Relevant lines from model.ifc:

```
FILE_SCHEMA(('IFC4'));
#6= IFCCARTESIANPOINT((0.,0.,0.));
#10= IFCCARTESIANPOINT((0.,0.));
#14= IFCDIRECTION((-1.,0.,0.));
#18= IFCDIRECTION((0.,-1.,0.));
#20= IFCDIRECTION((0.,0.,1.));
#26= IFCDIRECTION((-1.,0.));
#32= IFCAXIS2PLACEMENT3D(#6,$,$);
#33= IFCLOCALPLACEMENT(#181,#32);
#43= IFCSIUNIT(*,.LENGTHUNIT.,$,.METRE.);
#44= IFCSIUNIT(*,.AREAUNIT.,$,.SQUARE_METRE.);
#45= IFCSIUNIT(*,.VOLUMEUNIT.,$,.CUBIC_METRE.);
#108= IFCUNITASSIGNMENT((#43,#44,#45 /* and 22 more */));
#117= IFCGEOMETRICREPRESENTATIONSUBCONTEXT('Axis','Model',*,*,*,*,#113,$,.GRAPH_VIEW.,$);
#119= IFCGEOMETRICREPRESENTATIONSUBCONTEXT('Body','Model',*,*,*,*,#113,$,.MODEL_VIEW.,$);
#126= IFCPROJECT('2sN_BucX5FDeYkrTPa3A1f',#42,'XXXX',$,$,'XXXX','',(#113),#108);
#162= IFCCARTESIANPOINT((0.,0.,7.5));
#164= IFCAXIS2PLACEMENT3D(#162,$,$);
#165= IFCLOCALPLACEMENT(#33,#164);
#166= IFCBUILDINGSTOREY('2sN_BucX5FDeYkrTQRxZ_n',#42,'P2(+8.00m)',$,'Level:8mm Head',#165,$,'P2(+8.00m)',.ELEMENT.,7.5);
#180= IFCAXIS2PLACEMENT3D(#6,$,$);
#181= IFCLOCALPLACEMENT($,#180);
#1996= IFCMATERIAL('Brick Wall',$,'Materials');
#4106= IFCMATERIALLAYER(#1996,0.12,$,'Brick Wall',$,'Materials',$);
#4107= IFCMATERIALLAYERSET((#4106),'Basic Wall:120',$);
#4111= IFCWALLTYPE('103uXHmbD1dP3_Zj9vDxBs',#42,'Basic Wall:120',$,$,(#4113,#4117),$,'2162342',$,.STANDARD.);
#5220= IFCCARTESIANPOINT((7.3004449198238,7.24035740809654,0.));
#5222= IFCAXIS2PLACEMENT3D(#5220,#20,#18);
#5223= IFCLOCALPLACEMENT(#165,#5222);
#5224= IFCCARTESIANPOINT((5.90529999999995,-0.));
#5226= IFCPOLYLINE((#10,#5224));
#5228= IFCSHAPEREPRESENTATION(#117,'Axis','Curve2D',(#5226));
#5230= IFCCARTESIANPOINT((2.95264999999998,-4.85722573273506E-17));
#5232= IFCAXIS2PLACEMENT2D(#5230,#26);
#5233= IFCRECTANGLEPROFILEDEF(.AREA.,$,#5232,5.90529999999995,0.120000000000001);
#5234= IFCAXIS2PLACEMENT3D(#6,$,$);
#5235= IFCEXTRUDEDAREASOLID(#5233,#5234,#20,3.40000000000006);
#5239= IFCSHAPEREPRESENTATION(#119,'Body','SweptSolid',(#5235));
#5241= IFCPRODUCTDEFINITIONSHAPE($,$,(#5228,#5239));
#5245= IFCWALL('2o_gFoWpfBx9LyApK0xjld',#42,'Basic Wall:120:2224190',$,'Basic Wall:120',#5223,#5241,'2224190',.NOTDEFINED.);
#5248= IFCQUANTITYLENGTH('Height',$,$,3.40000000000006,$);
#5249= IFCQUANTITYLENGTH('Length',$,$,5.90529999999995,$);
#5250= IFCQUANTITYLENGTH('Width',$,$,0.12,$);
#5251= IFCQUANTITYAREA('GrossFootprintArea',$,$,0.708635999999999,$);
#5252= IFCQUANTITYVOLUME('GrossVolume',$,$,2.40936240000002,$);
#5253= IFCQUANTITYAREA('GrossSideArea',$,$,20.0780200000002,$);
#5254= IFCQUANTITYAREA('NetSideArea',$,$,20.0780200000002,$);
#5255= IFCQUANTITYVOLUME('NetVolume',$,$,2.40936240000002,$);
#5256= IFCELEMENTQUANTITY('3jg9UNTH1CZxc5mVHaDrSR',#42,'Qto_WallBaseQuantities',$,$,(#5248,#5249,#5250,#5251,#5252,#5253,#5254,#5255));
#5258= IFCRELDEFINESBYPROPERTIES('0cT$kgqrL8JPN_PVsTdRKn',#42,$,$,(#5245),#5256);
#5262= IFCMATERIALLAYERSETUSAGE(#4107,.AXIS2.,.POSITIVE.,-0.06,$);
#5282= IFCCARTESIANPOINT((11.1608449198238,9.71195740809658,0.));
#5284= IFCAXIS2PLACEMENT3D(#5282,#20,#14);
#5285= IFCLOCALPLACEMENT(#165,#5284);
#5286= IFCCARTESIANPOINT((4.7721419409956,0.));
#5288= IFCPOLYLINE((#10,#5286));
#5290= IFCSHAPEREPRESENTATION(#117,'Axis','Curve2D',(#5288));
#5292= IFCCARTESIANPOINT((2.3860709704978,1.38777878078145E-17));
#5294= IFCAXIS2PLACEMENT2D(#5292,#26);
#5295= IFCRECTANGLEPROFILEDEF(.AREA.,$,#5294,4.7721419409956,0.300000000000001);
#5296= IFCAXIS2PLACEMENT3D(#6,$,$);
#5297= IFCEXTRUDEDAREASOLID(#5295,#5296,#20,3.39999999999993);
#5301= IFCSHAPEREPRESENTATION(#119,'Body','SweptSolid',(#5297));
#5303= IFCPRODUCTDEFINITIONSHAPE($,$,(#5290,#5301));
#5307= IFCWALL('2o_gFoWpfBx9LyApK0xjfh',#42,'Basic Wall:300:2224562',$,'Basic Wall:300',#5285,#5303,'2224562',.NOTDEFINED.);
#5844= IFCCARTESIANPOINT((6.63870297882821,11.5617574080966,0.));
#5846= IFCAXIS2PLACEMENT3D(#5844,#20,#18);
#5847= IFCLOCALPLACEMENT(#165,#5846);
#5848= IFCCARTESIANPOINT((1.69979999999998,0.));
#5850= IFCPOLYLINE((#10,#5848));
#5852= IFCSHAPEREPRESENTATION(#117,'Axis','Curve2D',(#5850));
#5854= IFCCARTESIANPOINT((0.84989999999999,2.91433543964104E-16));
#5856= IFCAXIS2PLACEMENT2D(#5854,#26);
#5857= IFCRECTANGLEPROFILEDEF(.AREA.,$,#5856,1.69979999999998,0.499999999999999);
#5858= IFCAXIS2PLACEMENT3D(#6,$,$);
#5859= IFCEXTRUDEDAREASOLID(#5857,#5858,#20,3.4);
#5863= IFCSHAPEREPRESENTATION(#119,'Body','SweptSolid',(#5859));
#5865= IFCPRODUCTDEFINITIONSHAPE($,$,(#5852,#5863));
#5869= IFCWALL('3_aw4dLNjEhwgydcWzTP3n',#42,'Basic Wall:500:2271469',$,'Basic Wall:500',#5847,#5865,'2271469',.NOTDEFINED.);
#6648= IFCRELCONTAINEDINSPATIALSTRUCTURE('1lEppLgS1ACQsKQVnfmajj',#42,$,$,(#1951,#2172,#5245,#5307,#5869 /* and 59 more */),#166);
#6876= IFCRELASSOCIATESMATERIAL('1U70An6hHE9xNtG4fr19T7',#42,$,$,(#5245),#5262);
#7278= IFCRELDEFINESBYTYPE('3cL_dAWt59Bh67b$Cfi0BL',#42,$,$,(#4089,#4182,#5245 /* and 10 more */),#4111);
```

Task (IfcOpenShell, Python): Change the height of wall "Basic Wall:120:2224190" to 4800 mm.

```python
import ifcopenshell
import ifcopenshell.api.pset
import ifcopenshell.geom
import ifcopenshell.util.element
import ifcopenshell.util.representation
import ifcopenshell.util.shape
import ifcopenshell.util.unit

model = ifcopenshell.open("model.ifc")
unit_scale = ifcopenshell.util.unit.calculate_unit_scale(model)
area_scale = ifcopenshell.util.unit.calculate_unit_scale(model, "AREAUNIT")
volume_scale = ifcopenshell.util.unit.calculate_unit_scale(model, "VOLUMEUNIT")
settings = ifcopenshell.geom.settings()


def volume(element):
    """Net volume in cubic metres, openings subtracted."""
    shape = ifcopenshell.geom.create_shape(settings, element)
    return ifcopenshell.util.shape.get_volume(shape.geometry)


wall = model.by_guid("2o_gFoWpfBx9LyApK0xjld")
before = volume(wall)

body = ifcopenshell.util.representation.get_representation(wall, "Model", "Body")
solid = body.Items[0]
old_height = solid.Depth
solid.Depth = 4.8 / unit_scale
after = volume(wall)
thickness = 0.12  # wall thickness in metres

# Update the stored height, areas and volumes.
qto = model.by_id(ifcopenshell.util.element.get_pset(wall, "Qto_WallBaseQuantities", should_inherit=False)["id"])
ifcopenshell.api.pset.edit_qto(model, qto=qto, properties={
    "Height": solid.Depth,
    "GrossVolume": ifcopenshell.util.element.get_pset(wall, "Qto_WallBaseQuantities", "GrossVolume") * solid.Depth / old_height,
    "GrossSideArea": ifcopenshell.util.element.get_pset(wall, "Qto_WallBaseQuantities", "GrossSideArea") * solid.Depth / old_height,
    "NetSideArea": after / thickness / area_scale,
    "NetVolume": after / volume_scale,
})

print(f"height {old_height:g} -> {solid.Depth:g}, volume {before:.3f} -> {after:.3f} m3")

model.write("model_updated.ifc")
```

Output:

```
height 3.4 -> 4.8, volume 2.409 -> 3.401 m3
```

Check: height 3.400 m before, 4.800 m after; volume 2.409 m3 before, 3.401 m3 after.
